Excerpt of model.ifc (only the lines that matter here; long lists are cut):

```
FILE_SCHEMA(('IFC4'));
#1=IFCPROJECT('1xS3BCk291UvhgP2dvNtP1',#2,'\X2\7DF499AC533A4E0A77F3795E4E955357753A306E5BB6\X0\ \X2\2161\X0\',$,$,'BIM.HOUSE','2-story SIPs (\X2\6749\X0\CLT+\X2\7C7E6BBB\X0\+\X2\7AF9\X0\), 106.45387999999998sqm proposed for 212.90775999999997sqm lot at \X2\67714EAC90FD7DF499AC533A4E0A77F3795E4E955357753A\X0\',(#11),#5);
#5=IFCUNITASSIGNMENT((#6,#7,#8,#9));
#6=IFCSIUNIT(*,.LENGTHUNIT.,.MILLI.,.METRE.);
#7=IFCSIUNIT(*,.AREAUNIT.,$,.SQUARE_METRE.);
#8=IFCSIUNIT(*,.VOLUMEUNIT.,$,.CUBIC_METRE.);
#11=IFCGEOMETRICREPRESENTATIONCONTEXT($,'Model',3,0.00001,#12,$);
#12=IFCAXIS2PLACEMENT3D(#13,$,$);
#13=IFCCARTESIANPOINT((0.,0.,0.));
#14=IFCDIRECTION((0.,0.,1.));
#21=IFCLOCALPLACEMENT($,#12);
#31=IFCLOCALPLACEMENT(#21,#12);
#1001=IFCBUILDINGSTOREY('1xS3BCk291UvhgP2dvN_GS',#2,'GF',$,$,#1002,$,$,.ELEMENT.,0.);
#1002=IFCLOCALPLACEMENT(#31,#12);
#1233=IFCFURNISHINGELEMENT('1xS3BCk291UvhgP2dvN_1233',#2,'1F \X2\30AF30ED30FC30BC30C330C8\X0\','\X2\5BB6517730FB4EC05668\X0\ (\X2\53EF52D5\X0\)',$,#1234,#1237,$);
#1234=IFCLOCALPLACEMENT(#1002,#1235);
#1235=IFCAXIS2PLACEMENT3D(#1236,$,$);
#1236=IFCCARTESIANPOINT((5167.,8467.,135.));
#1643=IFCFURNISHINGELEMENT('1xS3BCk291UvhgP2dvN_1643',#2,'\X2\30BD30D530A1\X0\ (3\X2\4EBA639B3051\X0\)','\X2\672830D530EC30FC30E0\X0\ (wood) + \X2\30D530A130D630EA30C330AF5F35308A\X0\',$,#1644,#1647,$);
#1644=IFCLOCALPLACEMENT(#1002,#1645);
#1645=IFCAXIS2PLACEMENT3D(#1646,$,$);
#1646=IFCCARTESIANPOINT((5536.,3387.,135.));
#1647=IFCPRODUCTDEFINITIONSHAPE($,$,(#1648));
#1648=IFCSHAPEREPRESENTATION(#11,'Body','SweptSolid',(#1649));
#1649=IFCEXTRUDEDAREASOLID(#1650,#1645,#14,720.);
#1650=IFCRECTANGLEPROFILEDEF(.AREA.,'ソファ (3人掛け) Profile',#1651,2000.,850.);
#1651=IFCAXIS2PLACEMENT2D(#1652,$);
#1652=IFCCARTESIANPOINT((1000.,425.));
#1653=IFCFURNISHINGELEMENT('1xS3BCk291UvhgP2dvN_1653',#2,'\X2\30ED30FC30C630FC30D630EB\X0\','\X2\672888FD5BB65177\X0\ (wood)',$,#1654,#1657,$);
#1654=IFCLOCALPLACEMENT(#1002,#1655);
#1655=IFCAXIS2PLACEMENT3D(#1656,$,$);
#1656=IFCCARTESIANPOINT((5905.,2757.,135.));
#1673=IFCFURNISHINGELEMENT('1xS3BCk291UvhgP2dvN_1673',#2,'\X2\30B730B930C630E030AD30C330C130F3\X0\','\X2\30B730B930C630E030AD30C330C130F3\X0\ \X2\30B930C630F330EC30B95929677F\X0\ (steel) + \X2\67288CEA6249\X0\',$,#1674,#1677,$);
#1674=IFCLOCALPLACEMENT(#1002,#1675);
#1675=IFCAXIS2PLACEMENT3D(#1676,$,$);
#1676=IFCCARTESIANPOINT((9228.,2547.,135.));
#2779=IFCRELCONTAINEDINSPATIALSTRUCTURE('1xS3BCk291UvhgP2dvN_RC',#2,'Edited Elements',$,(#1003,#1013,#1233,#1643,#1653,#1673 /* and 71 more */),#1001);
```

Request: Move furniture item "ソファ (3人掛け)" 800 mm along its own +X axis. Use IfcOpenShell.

```python
import ifcopenshell
import ifcopenshell.api.geometry
import ifcopenshell.util.placement

model = ifcopenshell.open("model.ifc")

item = model.by_guid("1xS3BCk291UvhgP2dvN_1643")
matrix = ifcopenshell.util.placement.get_local_placement(item.ObjectPlacement)
matrix[:3, 3] += matrix[:3, 0] * 800.0
ifcopenshell.api.geometry.edit_object_placement(model, product=item, matrix=matrix, is_si=False)

print(ifcopenshell.util.placement.get_local_placement(item.ObjectPlacement).round(3) + 0.0)

model.write("model_updated.ifc")
```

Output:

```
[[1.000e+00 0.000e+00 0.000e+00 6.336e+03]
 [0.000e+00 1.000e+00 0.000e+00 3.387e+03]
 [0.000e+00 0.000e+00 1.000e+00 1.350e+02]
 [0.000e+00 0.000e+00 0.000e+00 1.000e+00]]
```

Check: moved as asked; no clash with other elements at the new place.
